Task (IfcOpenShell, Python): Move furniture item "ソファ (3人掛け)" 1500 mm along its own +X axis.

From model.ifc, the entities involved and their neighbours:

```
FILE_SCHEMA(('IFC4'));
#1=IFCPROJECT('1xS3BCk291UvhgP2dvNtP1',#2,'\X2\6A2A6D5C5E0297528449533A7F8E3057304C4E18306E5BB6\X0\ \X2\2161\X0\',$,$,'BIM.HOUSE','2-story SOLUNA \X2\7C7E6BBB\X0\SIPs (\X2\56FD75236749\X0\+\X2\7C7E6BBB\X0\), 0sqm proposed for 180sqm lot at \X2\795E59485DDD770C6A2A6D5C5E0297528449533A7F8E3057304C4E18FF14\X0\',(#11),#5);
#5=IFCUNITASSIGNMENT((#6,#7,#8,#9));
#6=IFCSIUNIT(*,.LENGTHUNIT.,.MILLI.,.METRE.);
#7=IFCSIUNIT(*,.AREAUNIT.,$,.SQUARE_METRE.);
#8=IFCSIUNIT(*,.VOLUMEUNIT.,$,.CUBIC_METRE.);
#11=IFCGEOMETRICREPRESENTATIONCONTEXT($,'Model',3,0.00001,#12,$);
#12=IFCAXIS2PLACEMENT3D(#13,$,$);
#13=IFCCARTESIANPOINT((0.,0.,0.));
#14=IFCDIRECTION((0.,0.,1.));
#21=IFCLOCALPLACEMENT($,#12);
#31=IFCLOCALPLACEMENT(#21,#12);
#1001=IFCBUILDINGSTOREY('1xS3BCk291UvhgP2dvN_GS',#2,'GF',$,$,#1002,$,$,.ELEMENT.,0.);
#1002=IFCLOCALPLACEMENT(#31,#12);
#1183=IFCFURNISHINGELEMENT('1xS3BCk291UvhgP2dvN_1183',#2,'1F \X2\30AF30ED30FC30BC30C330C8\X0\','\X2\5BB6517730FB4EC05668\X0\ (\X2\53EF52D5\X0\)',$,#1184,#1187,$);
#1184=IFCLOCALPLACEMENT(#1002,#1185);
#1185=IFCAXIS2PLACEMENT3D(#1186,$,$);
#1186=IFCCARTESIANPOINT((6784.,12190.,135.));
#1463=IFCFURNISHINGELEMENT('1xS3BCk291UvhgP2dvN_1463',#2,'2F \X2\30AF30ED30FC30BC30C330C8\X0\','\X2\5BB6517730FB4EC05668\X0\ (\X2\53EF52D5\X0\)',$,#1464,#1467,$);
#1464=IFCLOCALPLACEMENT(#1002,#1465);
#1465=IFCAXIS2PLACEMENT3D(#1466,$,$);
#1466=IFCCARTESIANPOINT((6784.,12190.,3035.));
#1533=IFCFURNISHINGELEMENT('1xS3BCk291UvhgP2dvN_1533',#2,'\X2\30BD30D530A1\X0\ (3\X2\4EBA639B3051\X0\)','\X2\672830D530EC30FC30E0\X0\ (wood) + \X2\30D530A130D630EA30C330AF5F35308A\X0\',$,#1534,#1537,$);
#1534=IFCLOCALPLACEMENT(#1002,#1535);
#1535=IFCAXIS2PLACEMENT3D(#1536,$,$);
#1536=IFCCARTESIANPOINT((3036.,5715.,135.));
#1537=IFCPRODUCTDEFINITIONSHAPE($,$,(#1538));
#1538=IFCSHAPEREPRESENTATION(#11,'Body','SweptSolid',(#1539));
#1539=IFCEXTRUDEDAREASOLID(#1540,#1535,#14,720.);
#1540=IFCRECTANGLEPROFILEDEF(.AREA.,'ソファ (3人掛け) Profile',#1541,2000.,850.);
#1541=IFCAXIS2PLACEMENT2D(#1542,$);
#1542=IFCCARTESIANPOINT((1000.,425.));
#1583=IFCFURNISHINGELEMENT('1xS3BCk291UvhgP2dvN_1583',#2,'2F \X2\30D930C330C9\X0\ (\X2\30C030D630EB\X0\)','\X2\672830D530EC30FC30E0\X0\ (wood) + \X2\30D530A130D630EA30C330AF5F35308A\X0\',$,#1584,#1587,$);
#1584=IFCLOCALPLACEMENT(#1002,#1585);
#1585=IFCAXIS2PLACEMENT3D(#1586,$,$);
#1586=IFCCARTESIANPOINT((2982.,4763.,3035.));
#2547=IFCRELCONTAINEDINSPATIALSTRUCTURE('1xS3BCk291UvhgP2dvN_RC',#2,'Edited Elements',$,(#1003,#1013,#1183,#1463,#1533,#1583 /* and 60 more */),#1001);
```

```python
import ifcopenshell
import ifcopenshell.api.geometry
import ifcopenshell.util.placement

model = ifcopenshell.open("model.ifc")

item = model.by_id(1533)
matrix = ifcopenshell.util.placement.get_local_placement(item.ObjectPlacement)
matrix[:3, 3] += matrix[:3, 0] * 1500.0
ifcopenshell.api.geometry.edit_object_placement(model, product=item, matrix=matrix, is_si=False)

print(ifcopenshell.util.placement.get_local_placement(item.ObjectPlacement).round(3) + 0.0)

model.write("model_rev.ifc")
```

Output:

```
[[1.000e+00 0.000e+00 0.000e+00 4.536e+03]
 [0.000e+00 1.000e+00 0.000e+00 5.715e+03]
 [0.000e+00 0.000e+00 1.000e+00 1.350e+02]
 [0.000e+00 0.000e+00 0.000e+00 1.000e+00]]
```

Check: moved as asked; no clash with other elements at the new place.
